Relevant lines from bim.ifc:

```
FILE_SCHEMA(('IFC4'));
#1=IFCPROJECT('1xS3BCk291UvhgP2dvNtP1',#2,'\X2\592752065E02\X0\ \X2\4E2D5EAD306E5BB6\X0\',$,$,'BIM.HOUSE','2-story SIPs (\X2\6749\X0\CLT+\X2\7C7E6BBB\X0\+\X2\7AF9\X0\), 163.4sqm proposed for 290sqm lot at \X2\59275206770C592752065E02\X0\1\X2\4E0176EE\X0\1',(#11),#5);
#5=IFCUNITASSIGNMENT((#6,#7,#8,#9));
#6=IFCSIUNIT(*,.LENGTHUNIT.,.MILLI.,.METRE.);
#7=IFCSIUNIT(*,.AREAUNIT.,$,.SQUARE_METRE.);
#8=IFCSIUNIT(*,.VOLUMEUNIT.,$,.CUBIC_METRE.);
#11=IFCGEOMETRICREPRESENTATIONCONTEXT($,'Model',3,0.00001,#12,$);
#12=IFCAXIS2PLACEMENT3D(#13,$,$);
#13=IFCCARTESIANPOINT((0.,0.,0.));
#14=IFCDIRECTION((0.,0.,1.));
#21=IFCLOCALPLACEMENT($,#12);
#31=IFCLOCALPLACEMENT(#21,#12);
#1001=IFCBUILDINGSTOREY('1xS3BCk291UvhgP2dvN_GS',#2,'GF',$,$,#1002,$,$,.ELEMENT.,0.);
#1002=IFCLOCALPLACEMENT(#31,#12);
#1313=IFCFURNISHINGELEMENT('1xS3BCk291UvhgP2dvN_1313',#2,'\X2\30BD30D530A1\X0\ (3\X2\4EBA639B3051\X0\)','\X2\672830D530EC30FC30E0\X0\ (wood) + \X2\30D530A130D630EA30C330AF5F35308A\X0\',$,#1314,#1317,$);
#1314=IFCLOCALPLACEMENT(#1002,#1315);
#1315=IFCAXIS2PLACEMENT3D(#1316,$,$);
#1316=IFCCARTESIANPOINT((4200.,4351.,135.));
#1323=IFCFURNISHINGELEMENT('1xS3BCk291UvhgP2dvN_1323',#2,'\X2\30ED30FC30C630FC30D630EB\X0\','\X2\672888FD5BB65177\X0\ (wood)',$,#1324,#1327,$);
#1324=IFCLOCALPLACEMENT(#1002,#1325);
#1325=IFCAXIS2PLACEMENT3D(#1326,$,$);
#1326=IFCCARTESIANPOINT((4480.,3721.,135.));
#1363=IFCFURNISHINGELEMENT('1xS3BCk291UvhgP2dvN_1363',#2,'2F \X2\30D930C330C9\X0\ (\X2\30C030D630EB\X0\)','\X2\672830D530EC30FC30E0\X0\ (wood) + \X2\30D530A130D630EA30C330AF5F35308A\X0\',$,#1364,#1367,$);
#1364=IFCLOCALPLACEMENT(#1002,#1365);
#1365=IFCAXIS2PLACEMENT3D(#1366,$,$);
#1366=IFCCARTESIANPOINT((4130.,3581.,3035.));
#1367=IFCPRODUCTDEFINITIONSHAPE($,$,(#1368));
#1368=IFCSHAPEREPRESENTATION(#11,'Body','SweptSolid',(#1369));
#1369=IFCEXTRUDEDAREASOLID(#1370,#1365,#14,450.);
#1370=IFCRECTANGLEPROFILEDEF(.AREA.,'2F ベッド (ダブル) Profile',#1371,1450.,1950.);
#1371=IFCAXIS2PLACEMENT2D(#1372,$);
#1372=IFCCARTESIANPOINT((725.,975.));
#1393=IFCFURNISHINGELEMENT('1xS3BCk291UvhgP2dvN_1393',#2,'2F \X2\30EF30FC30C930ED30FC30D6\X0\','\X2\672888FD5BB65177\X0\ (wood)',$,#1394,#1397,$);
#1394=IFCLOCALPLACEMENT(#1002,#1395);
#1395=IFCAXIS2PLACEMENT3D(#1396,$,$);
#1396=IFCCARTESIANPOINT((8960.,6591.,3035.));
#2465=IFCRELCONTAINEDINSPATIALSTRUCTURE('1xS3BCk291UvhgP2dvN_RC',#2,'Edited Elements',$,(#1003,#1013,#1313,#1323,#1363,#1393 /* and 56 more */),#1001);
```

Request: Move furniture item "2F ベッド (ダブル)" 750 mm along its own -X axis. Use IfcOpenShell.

```python
import ifcopenshell
import ifcopenshell.api.geometry
import ifcopenshell.util.placement

model = ifcopenshell.open("bim.ifc")

item = model.by_guid("1xS3BCk291UvhgP2dvN_1363")
matrix = ifcopenshell.util.placement.get_local_placement(item.ObjectPlacement)
matrix[:3, 3] -= matrix[:3, 0] * 750.0
ifcopenshell.api.geometry.edit_object_placement(model, product=item, matrix=matrix, is_si=False)

print(ifcopenshell.util.placement.get_local_placement(item.ObjectPlacement).round(3) + 0.0)

model.write("bim_edited.ifc")
```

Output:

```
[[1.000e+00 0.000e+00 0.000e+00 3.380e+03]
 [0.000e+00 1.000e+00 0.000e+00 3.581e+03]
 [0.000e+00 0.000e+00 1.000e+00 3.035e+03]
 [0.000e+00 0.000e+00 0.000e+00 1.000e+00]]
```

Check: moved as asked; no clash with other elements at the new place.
